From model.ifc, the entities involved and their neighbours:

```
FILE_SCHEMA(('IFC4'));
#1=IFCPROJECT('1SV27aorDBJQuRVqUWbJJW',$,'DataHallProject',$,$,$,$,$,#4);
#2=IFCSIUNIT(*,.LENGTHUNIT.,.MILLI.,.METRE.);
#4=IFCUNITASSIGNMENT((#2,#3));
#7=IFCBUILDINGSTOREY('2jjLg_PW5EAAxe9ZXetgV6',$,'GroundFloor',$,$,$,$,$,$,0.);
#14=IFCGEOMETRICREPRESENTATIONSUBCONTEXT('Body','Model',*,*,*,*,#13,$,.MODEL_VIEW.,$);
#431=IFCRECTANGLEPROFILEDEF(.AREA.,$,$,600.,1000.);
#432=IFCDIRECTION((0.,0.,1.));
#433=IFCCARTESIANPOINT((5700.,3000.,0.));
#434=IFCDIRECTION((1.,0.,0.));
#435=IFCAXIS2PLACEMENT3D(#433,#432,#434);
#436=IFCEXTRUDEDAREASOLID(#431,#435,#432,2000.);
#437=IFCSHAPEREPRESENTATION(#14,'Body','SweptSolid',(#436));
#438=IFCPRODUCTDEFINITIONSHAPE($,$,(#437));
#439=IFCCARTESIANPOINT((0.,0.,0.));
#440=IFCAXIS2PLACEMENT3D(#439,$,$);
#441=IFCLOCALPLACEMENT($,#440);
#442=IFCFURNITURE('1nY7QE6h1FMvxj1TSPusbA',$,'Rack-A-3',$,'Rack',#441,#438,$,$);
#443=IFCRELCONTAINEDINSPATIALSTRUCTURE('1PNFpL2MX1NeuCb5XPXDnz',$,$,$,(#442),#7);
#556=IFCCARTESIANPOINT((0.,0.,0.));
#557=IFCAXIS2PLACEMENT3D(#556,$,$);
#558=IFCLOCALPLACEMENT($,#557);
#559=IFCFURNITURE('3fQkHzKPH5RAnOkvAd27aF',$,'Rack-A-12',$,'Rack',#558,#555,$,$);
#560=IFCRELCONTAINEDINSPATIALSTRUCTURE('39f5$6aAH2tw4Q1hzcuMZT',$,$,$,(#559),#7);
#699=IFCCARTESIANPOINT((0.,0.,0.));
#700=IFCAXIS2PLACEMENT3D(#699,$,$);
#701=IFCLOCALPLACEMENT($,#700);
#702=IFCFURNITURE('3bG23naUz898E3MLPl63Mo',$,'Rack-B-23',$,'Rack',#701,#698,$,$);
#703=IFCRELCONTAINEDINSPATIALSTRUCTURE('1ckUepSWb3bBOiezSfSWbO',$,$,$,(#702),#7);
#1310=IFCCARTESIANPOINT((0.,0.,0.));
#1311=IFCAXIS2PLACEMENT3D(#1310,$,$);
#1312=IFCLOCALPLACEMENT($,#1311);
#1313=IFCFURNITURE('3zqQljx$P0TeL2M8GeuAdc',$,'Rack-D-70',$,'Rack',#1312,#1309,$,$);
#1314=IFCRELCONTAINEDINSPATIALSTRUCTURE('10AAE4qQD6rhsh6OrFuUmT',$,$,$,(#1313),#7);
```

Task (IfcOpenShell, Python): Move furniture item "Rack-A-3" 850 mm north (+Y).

```python
import ifcopenshell
import ifcopenshell.api.geometry
import ifcopenshell.util.placement

model = ifcopenshell.open("model.ifc")

item = model.by_guid("1nY7QE6h1FMvxj1TSPusbA")
matrix = ifcopenshell.util.placement.get_local_placement(item.ObjectPlacement)
matrix[1, 3] += 850.0
ifcopenshell.api.geometry.edit_object_placement(model, product=item, matrix=matrix, is_si=False)

print(ifcopenshell.util.placement.get_local_placement(item.ObjectPlacement).round(3) + 0.0)

model.write("model_edited.ifc")
```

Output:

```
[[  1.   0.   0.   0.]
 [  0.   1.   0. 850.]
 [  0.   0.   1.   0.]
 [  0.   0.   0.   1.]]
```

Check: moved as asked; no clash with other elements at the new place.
